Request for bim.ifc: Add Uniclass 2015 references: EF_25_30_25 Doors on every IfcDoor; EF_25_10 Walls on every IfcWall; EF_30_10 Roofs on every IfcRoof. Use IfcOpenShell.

First a look at what the model holds.

```python
import ifcopenshell

model = ifcopenshell.open("bim.ifc")
print(model.schema)
print("classifications:", [c.Name for c in model.by_type("IfcClassification")])
for ifc_class in ("IfcDoor", "IfcRoof", "IfcStair", "IfcWall", "IfcWindow"):
    print(ifc_class, len(model.by_type(ifc_class)))
```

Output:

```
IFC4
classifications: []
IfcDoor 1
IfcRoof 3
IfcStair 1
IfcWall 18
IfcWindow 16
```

```python
import ifcopenshell
import ifcopenshell.api.classification

model = ifcopenshell.open("bim.ifc")

system = ifcopenshell.api.classification.add_classification(model, classification="Uniclass 2015")

codes = {
    "IfcDoor": ("EF_25_30_25", "Doors"),
    "IfcWall": ("EF_25_10", "Walls"),
    "IfcRoof": ("EF_30_10", "Roofs"),
}
for ifc_class, (code, name) in codes.items():
    products = model.by_type(ifc_class)
    ifcopenshell.api.classification.add_reference(
        model, products=products, classification=system, identification=code, name=name
    )
    print(code, len(products))

model.write("bim_v2.ifc")
```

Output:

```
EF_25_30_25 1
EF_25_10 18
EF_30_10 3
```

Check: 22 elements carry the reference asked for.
